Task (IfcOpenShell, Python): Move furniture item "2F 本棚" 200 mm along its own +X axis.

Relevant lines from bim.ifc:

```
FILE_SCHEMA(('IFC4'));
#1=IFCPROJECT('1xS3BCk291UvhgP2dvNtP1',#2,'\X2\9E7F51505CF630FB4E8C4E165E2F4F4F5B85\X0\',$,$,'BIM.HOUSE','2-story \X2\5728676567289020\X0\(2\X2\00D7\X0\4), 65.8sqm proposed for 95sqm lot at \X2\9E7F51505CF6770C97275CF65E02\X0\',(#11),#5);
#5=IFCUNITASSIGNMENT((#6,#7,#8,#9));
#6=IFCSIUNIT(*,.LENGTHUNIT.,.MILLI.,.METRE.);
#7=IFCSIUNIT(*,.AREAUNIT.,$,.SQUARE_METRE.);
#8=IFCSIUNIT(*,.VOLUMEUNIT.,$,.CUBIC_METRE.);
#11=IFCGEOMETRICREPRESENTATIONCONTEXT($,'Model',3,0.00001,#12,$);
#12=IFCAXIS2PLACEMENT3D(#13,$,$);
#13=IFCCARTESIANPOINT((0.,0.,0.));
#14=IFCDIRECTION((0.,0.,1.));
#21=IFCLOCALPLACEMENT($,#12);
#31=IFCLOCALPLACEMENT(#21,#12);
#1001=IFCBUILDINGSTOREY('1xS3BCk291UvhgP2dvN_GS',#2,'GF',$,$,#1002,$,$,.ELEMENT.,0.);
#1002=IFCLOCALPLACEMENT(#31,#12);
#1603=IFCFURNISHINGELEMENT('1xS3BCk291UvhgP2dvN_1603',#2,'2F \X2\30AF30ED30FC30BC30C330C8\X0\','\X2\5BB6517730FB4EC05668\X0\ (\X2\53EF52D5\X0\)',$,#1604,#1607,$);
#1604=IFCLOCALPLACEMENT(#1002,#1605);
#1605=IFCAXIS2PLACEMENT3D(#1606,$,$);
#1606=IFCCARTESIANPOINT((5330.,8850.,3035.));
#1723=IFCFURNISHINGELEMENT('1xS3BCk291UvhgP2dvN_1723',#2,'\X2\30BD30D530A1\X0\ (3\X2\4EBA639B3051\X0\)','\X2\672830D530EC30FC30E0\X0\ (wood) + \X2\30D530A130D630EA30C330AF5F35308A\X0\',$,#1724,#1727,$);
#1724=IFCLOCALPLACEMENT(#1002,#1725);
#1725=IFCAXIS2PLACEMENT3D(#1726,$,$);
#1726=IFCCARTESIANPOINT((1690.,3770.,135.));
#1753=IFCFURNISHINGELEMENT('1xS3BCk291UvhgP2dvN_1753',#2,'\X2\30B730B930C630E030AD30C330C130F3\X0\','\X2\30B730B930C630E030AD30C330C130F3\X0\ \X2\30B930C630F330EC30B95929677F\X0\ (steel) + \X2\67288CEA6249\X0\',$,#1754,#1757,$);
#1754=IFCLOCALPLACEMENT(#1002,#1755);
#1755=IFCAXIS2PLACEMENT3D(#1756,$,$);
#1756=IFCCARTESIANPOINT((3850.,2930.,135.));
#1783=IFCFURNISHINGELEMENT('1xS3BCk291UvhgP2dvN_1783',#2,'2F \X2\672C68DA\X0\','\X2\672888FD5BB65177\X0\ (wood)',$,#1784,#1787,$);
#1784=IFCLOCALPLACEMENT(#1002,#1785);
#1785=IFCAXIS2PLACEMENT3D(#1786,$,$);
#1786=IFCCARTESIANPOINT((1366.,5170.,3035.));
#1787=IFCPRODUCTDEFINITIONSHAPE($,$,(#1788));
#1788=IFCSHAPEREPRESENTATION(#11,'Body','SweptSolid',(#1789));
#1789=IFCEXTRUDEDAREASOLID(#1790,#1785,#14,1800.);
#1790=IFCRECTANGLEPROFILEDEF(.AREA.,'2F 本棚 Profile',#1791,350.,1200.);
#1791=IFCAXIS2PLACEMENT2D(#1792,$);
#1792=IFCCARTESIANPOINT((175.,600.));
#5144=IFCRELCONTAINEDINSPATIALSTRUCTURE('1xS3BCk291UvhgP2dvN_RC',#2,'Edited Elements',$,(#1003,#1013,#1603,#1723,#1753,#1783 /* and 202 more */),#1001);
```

```python
import ifcopenshell
import ifcopenshell.api.geometry
import ifcopenshell.util.placement
import ifcopenshell.util.unit

model = ifcopenshell.open("bim.ifc")
unit_scale = ifcopenshell.util.unit.calculate_unit_scale(model)

item = model.by_id(1783)
matrix = ifcopenshell.util.placement.get_local_placement(item.ObjectPlacement)
matrix[:3, 3] += matrix[:3, 0] * 0.2 / unit_scale
ifcopenshell.api.geometry.edit_object_placement(model, product=item, matrix=matrix, is_si=False)

print(ifcopenshell.util.placement.get_local_placement(item.ObjectPlacement).round(3) + 0.0)

model.write("bim_rev.ifc")
```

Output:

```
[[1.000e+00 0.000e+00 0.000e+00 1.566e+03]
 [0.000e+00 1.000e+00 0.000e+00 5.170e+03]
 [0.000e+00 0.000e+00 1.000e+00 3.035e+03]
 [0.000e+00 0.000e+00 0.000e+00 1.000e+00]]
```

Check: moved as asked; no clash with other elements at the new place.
